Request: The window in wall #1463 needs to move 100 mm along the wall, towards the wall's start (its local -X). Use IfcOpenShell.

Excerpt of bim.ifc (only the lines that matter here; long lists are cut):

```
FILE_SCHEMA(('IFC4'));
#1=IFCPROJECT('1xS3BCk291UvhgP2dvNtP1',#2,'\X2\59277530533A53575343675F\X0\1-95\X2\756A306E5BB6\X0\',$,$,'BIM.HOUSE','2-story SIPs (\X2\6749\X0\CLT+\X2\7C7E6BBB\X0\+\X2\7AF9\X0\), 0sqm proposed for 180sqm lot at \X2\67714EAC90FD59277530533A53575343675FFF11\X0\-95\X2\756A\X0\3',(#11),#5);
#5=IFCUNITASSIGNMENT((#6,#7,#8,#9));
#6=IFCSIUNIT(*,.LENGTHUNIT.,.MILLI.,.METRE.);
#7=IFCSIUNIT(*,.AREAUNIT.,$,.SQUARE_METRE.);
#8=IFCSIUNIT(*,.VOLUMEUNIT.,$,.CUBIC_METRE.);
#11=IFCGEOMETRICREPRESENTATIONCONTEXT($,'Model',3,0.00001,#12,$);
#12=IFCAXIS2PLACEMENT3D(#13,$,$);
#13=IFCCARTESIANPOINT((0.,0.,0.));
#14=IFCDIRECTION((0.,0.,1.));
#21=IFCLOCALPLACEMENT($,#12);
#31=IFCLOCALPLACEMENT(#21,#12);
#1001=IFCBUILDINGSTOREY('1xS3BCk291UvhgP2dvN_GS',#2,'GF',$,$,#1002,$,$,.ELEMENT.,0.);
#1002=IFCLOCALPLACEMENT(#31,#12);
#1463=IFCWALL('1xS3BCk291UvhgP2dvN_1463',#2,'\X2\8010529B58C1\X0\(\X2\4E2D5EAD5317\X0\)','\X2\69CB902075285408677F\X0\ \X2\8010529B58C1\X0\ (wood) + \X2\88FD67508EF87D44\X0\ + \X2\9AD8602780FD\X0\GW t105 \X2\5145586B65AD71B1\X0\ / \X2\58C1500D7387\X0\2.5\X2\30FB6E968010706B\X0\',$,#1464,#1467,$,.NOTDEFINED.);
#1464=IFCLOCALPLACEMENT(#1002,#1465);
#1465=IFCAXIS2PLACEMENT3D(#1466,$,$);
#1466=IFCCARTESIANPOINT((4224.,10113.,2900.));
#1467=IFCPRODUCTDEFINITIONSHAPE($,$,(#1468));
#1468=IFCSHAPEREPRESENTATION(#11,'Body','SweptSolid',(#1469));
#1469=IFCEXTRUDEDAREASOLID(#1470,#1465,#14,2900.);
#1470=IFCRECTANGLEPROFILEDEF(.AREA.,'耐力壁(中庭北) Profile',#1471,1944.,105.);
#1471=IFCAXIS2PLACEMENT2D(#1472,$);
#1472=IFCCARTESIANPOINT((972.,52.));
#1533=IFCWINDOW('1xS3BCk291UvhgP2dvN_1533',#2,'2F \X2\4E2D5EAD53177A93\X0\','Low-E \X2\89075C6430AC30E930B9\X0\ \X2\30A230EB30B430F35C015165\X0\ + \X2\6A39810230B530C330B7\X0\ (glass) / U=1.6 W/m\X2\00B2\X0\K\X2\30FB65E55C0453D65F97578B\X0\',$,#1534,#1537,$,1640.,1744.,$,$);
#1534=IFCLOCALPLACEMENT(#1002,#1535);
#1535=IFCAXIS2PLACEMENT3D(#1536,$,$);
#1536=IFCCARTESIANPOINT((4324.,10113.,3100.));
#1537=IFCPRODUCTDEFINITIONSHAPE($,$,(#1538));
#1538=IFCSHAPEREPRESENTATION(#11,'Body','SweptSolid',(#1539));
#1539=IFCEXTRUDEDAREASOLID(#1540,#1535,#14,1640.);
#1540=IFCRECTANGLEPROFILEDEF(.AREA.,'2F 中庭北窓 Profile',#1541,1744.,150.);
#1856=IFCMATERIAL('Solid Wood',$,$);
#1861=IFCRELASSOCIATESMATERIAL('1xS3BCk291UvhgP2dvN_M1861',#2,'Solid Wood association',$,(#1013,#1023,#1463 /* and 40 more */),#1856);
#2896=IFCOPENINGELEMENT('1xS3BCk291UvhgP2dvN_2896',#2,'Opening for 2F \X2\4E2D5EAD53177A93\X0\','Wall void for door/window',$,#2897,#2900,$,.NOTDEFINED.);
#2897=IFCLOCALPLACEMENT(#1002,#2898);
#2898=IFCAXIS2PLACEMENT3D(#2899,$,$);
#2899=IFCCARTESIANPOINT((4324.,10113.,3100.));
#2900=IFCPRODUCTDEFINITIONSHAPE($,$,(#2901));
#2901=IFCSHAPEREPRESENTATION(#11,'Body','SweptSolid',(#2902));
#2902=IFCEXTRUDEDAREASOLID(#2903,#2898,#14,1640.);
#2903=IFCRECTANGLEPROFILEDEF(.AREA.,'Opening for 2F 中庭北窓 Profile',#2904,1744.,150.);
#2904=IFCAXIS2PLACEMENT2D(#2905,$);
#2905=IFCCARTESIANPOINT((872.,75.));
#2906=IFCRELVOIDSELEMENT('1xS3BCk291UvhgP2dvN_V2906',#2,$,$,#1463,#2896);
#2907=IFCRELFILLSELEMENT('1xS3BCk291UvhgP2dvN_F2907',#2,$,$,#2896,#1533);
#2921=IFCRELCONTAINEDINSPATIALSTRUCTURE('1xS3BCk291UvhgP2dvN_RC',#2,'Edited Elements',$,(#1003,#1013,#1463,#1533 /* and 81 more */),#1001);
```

```python
import ifcopenshell
import ifcopenshell.api.geometry
import ifcopenshell.util.placement
import ifcopenshell.util.unit

model = ifcopenshell.open("bim.ifc")
unit_scale = ifcopenshell.util.unit.calculate_unit_scale(model)

window = model.by_guid("1xS3BCk291UvhgP2dvN_1533")
opening = window.FillsVoids[0].RelatingOpeningElement
wall = opening.VoidsElements[0].RelatingBuildingElement

wall_matrix = ifcopenshell.util.placement.get_local_placement(wall.ObjectPlacement)
shift = wall_matrix[:3, 0] * -0.1 / unit_scale
before = ifcopenshell.util.placement.get_local_placement(window.ObjectPlacement)[:3, 3].copy()

# The window is not placed relative to its opening, so move both.
for product in (opening, window):
    matrix = ifcopenshell.util.placement.get_local_placement(product.ObjectPlacement)
    matrix[:3, 3] += shift
    ifcopenshell.api.geometry.edit_object_placement(model, product=product, matrix=matrix, is_si=False)

after = ifcopenshell.util.placement.get_local_placement(window.ObjectPlacement)[:3, 3]
print("window moved by", (after - before).round(3) + 0.0)

model.write("bim_updated.ifc")
```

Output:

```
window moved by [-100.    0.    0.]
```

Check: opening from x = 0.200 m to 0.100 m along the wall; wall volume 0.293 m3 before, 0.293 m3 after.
